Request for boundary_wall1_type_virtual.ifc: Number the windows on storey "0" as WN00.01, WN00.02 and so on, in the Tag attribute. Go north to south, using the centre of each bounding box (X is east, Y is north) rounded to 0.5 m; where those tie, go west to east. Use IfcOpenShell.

First a look at what the model holds.

```python
import ifcopenshell
import ifcopenshell.util.element
import ifcopenshell.util.placement

model = ifcopenshell.open("boundary_wall1_type_virtual.ifc")
print(model.schema)
storey = next(s for s in model.by_type("IfcBuildingStorey") if s.Name == "0")
windows = [e for e in ifcopenshell.util.element.get_decomposition(storey) if e.is_a("IfcWindow")]
for e in sorted(windows, key=lambda e: e.id()):
    origin = ifcopenshell.util.placement.get_local_placement(e.ObjectPlacement)[:3, 3]
    print(e.id(), e.Tag, e.Name, origin.round(2) + 0.0, sep=" | ")
```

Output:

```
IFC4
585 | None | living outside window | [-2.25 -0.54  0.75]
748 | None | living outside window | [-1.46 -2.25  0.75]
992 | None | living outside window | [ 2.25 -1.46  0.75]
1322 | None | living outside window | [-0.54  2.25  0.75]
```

```python
import ifcopenshell
import ifcopenshell.geom
import ifcopenshell.util.element
import ifcopenshell.util.shape

model = ifcopenshell.open("boundary_wall1_type_virtual.ifc")
settings = ifcopenshell.geom.settings()
settings.set("use-world-coords", True)


def centre(element):
    shape = ifcopenshell.geom.create_shape(settings, element)
    return ifcopenshell.util.shape.get_bbox_centroid(shape.geometry)


storey = next(s for s in model.by_type("IfcBuildingStorey") if s.Name == "0")
windows = [e for e in ifcopenshell.util.element.get_decomposition(storey) if e.is_a("IfcWindow")]

# Insertion points can sit at a corner or the storey origin, so sort by the geometry (in metres).
centres = {e: centre(e) for e in windows}
windows.sort(key=lambda e: (-round(centres[e][1] / 0.5), centres[e][0]))

for i, e in enumerate(windows, start=1):
    number = f"WN00.{i:02d}"
    e.Tag = number
    print(e.id(), number)

model.write("boundary_wall1_type_virtual_updated.ifc")
```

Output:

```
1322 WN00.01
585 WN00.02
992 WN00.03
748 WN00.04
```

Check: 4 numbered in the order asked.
